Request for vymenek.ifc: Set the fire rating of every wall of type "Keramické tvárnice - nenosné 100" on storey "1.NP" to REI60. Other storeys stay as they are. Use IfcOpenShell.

First a look at what the model holds.

```python
import ifcopenshell
import ifcopenshell.util.element

model = ifcopenshell.open("vymenek.ifc")
print(model.schema)
storey = next(s for s in model.by_type("IfcBuildingStorey") if s.Name == "1.NP")
walls = [e for e in ifcopenshell.util.element.get_decomposition(storey) if e.is_a("IfcWall")]
seen = {}
for e in walls:
    element_type = ifcopenshell.util.element.get_type(e)
    key = (element_type.Name if element_type != e and element_type else None, ifcopenshell.util.element.get_pset(e, "Pset_WallCommon", "FireRating"))
    seen[key] = seen.get(key, 0) + 1
for (name, value), count in sorted(seen.items(), key=str):
    print(count, "x", name, "|", value)
```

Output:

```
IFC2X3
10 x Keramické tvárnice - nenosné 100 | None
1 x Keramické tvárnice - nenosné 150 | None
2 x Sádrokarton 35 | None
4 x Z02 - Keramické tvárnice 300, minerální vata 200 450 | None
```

```python
import ifcopenshell
import ifcopenshell.api.pset
import ifcopenshell.util.element

model = ifcopenshell.open("vymenek.ifc")

storey = next(s for s in model.by_type("IfcBuildingStorey") if s.Name == "1.NP")
walls = [e for e in ifcopenshell.util.element.get_decomposition(storey) if e.is_a("IfcWall")]

count = 0
for e in walls:
    element_type = ifcopenshell.util.element.get_type(e)
    if element_type in (None, e) or element_type.Name != "Keramické tvárnice - nenosné 100":
        continue
    # add_pset returns the element's existing set when there is one.
    pset = ifcopenshell.api.pset.add_pset(model, product=e, name="Pset_WallCommon")
    ifcopenshell.api.pset.edit_pset(model, pset=pset, properties={"FireRating": "REI60"})
    count += 1

print(count, "walls updated")

model.write("vymenek_rev.ifc")
```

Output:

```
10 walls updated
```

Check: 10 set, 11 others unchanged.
